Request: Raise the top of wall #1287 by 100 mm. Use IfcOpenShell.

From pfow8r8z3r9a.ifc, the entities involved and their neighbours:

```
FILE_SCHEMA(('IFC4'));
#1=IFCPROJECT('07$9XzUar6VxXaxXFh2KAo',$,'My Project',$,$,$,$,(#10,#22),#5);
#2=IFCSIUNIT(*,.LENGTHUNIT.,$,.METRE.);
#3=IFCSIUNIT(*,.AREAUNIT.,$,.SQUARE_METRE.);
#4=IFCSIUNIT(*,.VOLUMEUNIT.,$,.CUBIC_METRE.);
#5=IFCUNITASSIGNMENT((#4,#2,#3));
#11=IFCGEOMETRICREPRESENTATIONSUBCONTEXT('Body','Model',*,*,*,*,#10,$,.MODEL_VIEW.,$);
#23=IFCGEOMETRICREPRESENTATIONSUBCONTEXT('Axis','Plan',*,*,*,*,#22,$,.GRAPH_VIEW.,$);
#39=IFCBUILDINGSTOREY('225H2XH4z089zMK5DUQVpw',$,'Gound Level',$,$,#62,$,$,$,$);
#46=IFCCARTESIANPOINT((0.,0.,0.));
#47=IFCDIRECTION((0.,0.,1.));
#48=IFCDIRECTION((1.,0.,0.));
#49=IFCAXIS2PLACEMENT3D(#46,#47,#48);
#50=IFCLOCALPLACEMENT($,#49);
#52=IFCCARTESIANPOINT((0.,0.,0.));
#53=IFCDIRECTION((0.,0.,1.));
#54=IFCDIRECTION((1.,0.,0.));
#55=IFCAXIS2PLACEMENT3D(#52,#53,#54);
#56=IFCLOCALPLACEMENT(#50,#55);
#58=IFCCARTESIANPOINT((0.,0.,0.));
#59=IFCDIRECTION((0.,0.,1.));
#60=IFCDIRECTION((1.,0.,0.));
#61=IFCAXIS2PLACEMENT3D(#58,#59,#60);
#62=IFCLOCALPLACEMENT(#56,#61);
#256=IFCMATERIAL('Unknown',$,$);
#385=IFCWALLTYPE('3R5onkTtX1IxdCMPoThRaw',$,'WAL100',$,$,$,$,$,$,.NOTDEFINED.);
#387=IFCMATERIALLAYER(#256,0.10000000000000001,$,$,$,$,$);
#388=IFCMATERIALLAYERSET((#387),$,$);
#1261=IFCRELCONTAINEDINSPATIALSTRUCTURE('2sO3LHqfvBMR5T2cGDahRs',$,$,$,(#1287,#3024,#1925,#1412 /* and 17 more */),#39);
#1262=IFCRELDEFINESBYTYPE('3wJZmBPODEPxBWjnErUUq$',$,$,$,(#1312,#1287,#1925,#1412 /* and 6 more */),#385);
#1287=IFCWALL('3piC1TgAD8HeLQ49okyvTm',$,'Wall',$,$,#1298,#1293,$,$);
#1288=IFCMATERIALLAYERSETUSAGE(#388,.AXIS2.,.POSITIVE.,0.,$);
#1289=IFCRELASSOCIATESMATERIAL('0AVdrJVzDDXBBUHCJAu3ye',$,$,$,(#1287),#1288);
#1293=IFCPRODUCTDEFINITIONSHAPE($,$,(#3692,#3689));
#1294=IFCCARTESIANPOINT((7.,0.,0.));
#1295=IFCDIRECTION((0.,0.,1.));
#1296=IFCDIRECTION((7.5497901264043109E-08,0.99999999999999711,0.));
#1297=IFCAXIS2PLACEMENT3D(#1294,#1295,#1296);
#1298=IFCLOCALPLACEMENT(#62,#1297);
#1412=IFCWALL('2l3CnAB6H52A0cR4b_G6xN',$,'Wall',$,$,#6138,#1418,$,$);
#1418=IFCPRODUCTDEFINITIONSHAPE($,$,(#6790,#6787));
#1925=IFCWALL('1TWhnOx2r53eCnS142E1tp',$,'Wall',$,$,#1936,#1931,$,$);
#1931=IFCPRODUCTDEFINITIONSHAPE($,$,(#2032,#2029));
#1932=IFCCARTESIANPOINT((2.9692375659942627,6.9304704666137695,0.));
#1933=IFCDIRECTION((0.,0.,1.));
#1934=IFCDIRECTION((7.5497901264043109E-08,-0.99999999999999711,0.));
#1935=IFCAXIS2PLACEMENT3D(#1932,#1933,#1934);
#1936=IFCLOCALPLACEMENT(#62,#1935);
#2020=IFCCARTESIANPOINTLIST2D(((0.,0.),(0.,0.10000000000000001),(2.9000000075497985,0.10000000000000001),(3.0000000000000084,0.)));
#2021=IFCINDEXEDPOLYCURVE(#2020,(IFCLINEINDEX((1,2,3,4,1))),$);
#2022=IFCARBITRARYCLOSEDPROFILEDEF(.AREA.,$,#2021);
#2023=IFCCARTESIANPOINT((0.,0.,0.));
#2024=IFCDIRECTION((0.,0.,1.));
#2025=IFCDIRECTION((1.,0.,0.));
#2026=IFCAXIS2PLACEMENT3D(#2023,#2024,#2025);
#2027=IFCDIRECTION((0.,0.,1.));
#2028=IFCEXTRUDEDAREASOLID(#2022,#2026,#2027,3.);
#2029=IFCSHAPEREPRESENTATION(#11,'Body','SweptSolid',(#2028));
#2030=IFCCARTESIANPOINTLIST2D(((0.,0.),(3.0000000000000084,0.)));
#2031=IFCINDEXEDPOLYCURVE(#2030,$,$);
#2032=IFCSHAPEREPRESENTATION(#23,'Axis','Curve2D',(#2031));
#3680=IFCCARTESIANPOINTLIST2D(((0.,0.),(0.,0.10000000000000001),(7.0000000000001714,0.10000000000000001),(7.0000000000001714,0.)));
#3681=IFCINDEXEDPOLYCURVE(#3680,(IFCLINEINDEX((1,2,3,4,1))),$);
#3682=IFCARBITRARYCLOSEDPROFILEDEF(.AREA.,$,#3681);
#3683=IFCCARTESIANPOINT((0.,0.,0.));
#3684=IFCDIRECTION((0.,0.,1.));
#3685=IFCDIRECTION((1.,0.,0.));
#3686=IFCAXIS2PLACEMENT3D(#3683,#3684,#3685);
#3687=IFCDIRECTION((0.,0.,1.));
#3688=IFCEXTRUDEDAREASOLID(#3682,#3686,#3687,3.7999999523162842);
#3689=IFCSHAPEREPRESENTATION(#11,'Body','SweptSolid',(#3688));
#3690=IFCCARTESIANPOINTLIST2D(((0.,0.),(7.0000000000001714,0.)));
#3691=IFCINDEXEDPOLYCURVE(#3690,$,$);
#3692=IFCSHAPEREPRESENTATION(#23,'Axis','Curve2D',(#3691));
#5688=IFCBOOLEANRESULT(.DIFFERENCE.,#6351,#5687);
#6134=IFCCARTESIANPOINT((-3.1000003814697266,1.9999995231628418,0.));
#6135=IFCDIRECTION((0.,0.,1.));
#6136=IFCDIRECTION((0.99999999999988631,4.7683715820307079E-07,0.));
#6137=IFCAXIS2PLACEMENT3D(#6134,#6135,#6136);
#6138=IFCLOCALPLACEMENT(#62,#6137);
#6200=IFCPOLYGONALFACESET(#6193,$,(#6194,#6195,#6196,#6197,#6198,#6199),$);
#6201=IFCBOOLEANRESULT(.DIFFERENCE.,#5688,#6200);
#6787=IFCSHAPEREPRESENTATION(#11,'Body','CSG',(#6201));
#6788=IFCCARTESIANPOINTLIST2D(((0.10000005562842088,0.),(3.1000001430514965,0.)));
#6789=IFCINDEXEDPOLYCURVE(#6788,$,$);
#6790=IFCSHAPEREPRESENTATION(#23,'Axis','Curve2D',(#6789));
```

```python
import ifcopenshell
import ifcopenshell.geom
import ifcopenshell.util.representation
import ifcopenshell.util.shape
import ifcopenshell.util.unit

model = ifcopenshell.open("pfow8r8z3r9a.ifc")
unit_scale = ifcopenshell.util.unit.calculate_unit_scale(model)
settings = ifcopenshell.geom.settings()


def volume(element):
    """Net volume in cubic metres, openings subtracted."""
    shape = ifcopenshell.geom.create_shape(settings, element)
    return ifcopenshell.util.shape.get_volume(shape.geometry)


wall = model.by_id(1287)
before = volume(wall)

body = ifcopenshell.util.representation.get_representation(wall, "Model", "Body")
solid = body.Items[0]
old_height = solid.Depth
solid.Depth += 0.1 / unit_scale
after = volume(wall)

print(f"height {old_height:g} -> {solid.Depth:g}, volume {before:.3f} -> {after:.3f} m3")

model.write("pfow8r8z3r9a_v2.ifc")
```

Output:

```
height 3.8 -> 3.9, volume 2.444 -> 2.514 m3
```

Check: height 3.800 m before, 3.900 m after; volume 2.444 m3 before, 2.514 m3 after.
